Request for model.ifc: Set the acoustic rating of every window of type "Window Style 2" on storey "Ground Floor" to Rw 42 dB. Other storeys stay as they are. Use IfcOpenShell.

First a look at what the model holds.

```python
import ifcopenshell
import ifcopenshell.util.element

model = ifcopenshell.open("model.ifc")
print(model.schema)
storey = next(s for s in model.by_type("IfcBuildingStorey") if s.Name == "Ground Floor")
windows = [e for e in ifcopenshell.util.element.get_decomposition(storey) if e.is_a("IfcWindow")]
seen = {}
for e in windows:
    element_type = ifcopenshell.util.element.get_type(e)
    key = (element_type.Name if element_type != e and element_type else None, ifcopenshell.util.element.get_pset(e, "Pset_WindowCommon", "AcousticRating"))
    seen[key] = seen.get(key, 0) + 1
for (name, value), count in sorted(seen.items(), key=str):
    print(count, "x", name, "|", value)
```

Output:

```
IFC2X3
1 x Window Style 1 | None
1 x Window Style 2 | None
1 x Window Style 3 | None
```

```python
import ifcopenshell
import ifcopenshell.api.pset
import ifcopenshell.util.element

model = ifcopenshell.open("model.ifc")

storey = next(s for s in model.by_type("IfcBuildingStorey") if s.Name == "Ground Floor")
windows = [e for e in ifcopenshell.util.element.get_decomposition(storey) if e.is_a("IfcWindow")]

count = 0
for e in windows:
    element_type = ifcopenshell.util.element.get_type(e)
    if element_type in (None, e) or element_type.Name != "Window Style 2":
        continue
    # add_pset returns the element's existing set when there is one.
    pset = ifcopenshell.api.pset.add_pset(model, product=e, name="Pset_WindowCommon")
    ifcopenshell.api.pset.edit_pset(model, pset=pset, properties={"AcousticRating": "Rw 42 dB"})
    count += 1

print(count, "windows updated")

model.write("model-out.ifc")
```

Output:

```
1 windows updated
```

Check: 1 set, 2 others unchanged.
